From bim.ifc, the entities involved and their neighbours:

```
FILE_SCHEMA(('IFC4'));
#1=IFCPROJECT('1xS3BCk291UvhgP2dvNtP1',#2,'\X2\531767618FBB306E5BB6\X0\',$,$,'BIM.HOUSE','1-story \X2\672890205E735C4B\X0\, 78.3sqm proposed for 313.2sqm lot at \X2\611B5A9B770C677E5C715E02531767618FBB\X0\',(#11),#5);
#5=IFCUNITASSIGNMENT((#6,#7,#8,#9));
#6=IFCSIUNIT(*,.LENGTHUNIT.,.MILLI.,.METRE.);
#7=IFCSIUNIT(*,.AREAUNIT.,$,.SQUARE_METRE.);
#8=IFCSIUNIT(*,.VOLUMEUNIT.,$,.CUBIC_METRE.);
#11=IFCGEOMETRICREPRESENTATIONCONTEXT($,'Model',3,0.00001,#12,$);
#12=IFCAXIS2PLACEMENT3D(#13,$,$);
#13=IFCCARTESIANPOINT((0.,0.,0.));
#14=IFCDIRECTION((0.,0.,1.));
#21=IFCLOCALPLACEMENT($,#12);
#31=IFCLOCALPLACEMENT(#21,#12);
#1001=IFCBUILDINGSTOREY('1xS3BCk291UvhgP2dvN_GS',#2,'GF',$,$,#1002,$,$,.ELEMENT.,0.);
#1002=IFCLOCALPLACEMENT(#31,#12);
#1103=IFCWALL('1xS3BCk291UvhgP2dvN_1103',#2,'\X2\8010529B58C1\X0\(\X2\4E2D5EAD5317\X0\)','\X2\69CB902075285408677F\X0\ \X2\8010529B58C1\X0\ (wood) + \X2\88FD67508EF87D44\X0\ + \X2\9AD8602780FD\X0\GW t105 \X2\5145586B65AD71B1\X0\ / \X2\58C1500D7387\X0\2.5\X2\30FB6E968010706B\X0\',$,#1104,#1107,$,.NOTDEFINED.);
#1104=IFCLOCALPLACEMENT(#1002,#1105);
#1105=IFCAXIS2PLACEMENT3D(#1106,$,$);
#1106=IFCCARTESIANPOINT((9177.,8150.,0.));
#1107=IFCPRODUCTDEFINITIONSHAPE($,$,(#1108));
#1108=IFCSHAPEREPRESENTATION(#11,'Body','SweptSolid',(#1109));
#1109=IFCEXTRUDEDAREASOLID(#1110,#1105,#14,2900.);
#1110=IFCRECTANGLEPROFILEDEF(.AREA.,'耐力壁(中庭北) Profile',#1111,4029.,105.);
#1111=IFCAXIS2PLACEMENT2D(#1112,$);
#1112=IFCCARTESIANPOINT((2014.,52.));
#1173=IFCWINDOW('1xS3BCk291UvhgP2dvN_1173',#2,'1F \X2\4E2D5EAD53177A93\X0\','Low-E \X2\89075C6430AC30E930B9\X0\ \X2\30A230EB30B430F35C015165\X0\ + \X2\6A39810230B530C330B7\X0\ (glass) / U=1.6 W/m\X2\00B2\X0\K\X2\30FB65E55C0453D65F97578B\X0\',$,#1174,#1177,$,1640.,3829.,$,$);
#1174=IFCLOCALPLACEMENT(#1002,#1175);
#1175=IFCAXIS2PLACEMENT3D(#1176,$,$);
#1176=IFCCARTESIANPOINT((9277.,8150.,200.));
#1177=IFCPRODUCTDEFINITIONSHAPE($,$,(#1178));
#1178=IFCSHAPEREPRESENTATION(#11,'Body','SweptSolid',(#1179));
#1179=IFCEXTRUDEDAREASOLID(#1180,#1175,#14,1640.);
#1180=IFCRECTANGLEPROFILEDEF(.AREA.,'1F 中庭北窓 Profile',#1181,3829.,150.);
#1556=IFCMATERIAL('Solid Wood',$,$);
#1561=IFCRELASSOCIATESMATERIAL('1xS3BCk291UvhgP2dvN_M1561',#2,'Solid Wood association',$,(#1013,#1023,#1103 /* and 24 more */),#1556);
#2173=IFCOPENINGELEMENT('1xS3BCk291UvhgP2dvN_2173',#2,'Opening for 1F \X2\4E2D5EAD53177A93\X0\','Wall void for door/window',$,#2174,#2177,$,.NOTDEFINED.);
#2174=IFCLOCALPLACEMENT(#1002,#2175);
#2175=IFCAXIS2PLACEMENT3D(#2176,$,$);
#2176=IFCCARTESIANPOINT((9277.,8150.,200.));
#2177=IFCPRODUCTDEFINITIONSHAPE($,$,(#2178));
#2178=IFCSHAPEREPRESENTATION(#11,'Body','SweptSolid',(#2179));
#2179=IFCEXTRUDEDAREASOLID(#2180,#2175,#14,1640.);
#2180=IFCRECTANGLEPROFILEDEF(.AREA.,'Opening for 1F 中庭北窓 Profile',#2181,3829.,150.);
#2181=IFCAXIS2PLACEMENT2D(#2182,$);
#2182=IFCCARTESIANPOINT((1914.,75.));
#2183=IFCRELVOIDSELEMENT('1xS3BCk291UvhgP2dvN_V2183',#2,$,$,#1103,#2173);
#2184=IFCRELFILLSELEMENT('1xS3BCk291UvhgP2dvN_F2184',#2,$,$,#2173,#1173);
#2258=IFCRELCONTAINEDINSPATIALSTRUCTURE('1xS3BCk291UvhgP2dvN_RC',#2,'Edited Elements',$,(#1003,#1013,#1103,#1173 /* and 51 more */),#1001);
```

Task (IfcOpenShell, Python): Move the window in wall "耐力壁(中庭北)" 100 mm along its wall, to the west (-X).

```python
import ifcopenshell
import ifcopenshell.api.geometry
import ifcopenshell.util.placement
import ifcopenshell.util.unit

model = ifcopenshell.open("bim.ifc")
unit_scale = ifcopenshell.util.unit.calculate_unit_scale(model)

window = model.by_guid("1xS3BCk291UvhgP2dvN_1173")
opening = window.FillsVoids[0].RelatingOpeningElement
wall = opening.VoidsElements[0].RelatingBuildingElement

wall_matrix = ifcopenshell.util.placement.get_local_placement(wall.ObjectPlacement)
shift = wall_matrix[:3, 0] * -0.1 / unit_scale
before = ifcopenshell.util.placement.get_local_placement(window.ObjectPlacement)[:3, 3].copy()

# The window is not placed relative to its opening, so move both.
for product in (opening, window):
    matrix = ifcopenshell.util.placement.get_local_placement(product.ObjectPlacement)
    matrix[:3, 3] += shift
    ifcopenshell.api.geometry.edit_object_placement(model, product=product, matrix=matrix, is_si=False)

after = ifcopenshell.util.placement.get_local_placement(window.ObjectPlacement)[:3, 3]
print("window moved by", (after - before).round(3) + 0.0)

model.write("bim_edited.ifc")
```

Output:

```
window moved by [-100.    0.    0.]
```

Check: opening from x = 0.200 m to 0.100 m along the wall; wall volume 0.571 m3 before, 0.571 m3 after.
